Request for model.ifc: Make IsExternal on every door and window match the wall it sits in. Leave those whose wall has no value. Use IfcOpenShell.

First a look at what the model holds.

```python
import ifcopenshell
import ifcopenshell.util.element

model = ifcopenshell.open("model.ifc")
print(model.schema)
seen = {}
for e in model.by_type("IfcDoor") + model.by_type("IfcWindow"):
    if not e.FillsVoids:
        continue
    host = e.FillsVoids[0].RelatingOpeningElement.VoidsElements[0].RelatingBuildingElement
    own = ifcopenshell.util.element.get_pset(e, f"Pset_{e.is_a()[3:].removesuffix('StandardCase')}Common", "IsExternal")
    wall = ifcopenshell.util.element.get_pset(host, "Pset_WallCommon", "IsExternal")
    seen[e.is_a(), own, wall] = seen.get((e.is_a(), own, wall), 0) + 1
for (cls, own, wall), count in sorted(seen.items(), key=str):
    print(count, cls, "IsExternal:", own, "| host wall:", wall)
```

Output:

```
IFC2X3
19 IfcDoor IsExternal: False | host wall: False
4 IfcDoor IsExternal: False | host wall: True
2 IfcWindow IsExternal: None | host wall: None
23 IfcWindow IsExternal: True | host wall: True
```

```python
import ifcopenshell
import ifcopenshell.api.pset
import ifcopenshell.util.element

model = ifcopenshell.open("model.ifc")

count = 0
for ifc_class, pset_name in (("IfcDoor", "Pset_DoorCommon"), ("IfcWindow", "Pset_WindowCommon")):
    for e in model.by_type(ifc_class):
        if not e.FillsVoids:
            continue
        host = e.FillsVoids[0].RelatingOpeningElement.VoidsElements[0].RelatingBuildingElement
        external = ifcopenshell.util.element.get_pset(host, "Pset_WallCommon", "IsExternal")
        if external is None or ifcopenshell.util.element.get_pset(e, pset_name, "IsExternal") == external:
            continue
        found = ifcopenshell.util.element.get_pset(e, pset_name, should_inherit=False)
        if found:
            pset = model.by_id(found["id"])
            if len(ifcopenshell.util.element.get_elements_by_pset(pset)) > 1:
                pset = ifcopenshell.api.pset.unshare_pset(model, products=[e], pset=pset)[0]
        else:
            pset = ifcopenshell.api.pset.add_pset(model, product=e, name=pset_name)
        ifcopenshell.api.pset.edit_pset(model, pset=pset, properties={"IsExternal": external})
        count += 1

print(count, "updated")

model.write("model_rev.ifc")
```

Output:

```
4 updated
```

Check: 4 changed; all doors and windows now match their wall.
